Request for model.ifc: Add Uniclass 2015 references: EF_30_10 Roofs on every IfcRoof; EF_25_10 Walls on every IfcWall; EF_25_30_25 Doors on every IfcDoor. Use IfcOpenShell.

First a look at what the model holds.

```python
import ifcopenshell

model = ifcopenshell.open("model.ifc")
print(model.schema)
print("classifications:", [c.Name for c in model.by_type("IfcClassification")])
for ifc_class in ("IfcDoor", "IfcRoof", "IfcStair", "IfcWall", "IfcWindow"):
    print(ifc_class, len(model.by_type(ifc_class)))
```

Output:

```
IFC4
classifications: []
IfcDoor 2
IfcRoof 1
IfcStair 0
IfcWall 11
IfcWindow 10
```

```python
import ifcopenshell
import ifcopenshell.api.classification

model = ifcopenshell.open("model.ifc")

system = ifcopenshell.api.classification.add_classification(model, classification="Uniclass 2015")

codes = {
    "IfcRoof": ("EF_30_10", "Roofs"),
    "IfcWall": ("EF_25_10", "Walls"),
    "IfcDoor": ("EF_25_30_25", "Doors"),
}
for ifc_class, (code, name) in codes.items():
    products = model.by_type(ifc_class)
    ifcopenshell.api.classification.add_reference(
        model, products=products, classification=system, identification=code, name=name
    )
    print(code, len(products))

model.write("model_edited.ifc")
```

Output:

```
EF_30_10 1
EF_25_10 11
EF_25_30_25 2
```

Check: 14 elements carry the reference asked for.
